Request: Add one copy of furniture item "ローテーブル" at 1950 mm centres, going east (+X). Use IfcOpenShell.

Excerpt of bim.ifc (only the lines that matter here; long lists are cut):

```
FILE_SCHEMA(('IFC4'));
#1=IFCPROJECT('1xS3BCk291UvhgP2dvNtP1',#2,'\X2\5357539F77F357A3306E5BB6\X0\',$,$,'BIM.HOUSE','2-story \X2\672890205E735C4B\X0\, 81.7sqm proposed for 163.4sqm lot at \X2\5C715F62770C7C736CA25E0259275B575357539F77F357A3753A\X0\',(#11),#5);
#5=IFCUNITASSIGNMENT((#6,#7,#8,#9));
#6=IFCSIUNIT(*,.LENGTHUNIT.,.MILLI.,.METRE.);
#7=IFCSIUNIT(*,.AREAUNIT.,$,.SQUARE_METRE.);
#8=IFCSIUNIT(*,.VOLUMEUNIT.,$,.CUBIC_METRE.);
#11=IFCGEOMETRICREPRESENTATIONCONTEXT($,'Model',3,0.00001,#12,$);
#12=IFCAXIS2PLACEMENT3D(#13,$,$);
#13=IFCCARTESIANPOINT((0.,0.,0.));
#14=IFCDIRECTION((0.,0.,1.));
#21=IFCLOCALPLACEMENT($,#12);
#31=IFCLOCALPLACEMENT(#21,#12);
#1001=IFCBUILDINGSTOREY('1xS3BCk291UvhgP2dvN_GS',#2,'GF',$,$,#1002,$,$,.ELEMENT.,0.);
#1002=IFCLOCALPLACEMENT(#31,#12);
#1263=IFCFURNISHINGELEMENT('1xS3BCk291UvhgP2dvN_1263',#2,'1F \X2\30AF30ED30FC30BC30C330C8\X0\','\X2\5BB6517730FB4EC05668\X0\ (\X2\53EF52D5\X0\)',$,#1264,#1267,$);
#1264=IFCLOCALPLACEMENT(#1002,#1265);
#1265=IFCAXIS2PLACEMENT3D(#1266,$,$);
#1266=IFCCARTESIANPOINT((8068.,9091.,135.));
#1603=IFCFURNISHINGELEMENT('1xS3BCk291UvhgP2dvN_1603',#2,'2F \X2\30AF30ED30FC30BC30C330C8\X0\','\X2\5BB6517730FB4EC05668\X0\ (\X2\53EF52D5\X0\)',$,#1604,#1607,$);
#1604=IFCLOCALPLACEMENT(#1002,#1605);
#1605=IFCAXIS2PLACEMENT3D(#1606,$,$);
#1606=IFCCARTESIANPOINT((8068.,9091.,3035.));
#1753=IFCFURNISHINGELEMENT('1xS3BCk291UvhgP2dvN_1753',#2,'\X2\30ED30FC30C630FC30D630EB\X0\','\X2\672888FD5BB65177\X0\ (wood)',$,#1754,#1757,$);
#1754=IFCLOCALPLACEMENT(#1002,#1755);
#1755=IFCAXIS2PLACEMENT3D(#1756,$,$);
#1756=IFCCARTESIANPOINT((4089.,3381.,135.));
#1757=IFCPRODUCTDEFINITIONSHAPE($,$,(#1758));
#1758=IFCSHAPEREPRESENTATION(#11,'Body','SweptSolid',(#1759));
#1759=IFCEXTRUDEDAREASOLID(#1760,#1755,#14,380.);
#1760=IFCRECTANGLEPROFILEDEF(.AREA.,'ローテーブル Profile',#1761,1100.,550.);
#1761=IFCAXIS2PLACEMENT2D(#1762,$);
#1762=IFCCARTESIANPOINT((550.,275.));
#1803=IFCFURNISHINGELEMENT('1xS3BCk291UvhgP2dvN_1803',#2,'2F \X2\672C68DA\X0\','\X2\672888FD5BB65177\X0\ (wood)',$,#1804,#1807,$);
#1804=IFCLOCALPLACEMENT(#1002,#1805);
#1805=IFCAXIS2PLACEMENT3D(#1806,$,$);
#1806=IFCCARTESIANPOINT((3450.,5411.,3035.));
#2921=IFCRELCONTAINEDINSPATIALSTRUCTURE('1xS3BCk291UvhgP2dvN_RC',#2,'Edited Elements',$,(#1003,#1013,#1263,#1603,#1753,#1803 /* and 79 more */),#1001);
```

```python
import numpy as np
import ifcopenshell
import ifcopenshell.api.geometry
import ifcopenshell.api.root
import ifcopenshell.util.element
import ifcopenshell.util.placement

model = ifcopenshell.open("bim.ifc")


def reuse_history(source, copy):
    """copy_class also copies each property set's owner history, people and application; keep the originals."""
    for rel in copy.IsDefinedBy:
        if rel.is_a("IfcRelDefinesByProperties") and (history := rel.RelatingPropertyDefinition.OwnerHistory):
            rel.RelatingPropertyDefinition.OwnerHistory = source.OwnerHistory
            ifcopenshell.util.element.remove_deep2(model, history)


source = model.by_guid("1xS3BCk291UvhgP2dvN_1753")
base = ifcopenshell.util.placement.get_local_placement(source.ObjectPlacement)
step = np.array([1.0, 0.0, 0.0]) * 1950.0

for i in range(1, 2):
    copy = ifcopenshell.api.root.copy_class(model, product=source)
    copy.Representation = ifcopenshell.util.element.copy_deep(
        model, source.Representation, exclude=["IfcGeometricRepresentationContext", "IfcRepresentationMap"]
    )
    reuse_history(source, copy)
    matrix = base.copy()
    matrix[:3, 3] += i * step
    print("added at", matrix[:3, 3].round(3) + 0.0)
    ifcopenshell.api.geometry.edit_object_placement(model, product=copy, matrix=matrix, is_si=False)

model.write("bim_v2.ifc")
```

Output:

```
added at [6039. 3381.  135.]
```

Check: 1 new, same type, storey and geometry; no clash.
